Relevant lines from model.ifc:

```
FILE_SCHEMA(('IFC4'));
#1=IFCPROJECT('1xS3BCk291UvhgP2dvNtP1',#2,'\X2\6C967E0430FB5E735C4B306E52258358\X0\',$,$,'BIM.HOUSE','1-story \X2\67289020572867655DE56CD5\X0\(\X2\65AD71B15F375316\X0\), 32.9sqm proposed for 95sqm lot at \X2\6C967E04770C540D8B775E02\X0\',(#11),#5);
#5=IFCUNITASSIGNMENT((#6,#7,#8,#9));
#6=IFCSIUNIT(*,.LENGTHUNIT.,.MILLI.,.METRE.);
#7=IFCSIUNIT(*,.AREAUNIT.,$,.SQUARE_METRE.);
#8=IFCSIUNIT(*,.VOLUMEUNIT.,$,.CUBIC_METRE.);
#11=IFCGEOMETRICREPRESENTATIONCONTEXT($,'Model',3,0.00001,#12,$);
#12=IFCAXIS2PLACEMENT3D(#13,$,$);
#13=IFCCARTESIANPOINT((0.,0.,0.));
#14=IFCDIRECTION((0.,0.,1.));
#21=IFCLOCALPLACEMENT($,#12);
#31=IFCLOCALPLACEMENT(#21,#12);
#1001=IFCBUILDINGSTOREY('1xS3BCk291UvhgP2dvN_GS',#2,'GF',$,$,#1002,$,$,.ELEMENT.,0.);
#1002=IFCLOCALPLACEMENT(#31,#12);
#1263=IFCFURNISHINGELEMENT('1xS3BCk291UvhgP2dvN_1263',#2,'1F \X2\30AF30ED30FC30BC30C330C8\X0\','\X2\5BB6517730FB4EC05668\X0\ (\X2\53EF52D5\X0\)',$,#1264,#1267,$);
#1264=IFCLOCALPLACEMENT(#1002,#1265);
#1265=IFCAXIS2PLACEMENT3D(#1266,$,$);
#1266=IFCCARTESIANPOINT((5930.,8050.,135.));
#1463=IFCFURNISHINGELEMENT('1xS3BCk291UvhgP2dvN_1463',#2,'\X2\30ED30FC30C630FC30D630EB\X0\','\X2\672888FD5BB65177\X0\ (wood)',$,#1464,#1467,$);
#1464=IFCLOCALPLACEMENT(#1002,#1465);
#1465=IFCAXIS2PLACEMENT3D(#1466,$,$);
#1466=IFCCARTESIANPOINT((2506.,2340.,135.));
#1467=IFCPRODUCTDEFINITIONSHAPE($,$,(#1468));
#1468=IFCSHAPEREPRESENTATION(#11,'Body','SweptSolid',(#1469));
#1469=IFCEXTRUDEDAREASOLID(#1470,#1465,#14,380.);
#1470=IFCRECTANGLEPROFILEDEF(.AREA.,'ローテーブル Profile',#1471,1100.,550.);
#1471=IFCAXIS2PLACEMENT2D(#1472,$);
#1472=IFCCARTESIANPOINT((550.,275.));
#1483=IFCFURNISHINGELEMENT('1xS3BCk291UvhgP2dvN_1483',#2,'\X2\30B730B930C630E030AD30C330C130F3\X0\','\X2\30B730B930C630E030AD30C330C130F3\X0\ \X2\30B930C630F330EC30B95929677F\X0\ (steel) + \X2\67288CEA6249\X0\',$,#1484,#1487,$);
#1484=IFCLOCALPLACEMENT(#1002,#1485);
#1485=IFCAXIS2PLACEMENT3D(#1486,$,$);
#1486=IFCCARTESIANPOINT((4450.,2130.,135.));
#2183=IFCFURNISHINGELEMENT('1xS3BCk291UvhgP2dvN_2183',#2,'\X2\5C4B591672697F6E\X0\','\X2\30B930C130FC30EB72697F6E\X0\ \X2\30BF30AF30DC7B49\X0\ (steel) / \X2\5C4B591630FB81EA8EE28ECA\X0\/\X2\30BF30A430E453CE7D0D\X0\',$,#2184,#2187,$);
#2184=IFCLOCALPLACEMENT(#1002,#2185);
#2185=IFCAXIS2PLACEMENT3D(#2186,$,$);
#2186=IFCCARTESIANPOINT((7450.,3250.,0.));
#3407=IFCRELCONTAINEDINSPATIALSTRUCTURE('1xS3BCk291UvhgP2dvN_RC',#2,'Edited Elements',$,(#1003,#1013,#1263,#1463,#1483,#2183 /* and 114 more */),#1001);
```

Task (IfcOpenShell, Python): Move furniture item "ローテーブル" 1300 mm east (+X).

```python
import ifcopenshell
import ifcopenshell.api.geometry
import ifcopenshell.util.placement
import ifcopenshell.util.unit

model = ifcopenshell.open("model.ifc")
unit_scale = ifcopenshell.util.unit.calculate_unit_scale(model)

item = model.by_id(1463)
matrix = ifcopenshell.util.placement.get_local_placement(item.ObjectPlacement)
matrix[0, 3] += 1.3 / unit_scale
ifcopenshell.api.geometry.edit_object_placement(model, product=item, matrix=matrix, is_si=False)

print(ifcopenshell.util.placement.get_local_placement(item.ObjectPlacement).round(3) + 0.0)

model.write("model_rev.ifc")
```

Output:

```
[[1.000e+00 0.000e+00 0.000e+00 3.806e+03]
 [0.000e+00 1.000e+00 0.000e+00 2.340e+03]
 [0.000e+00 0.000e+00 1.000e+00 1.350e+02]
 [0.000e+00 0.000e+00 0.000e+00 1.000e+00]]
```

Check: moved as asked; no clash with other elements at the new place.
